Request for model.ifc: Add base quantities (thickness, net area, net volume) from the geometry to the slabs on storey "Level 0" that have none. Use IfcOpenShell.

First a look at what the model holds.

```python
import ifcopenshell
import ifcopenshell.util.element
import ifcopenshell.util.unit

model = ifcopenshell.open("model.ifc")
print(model.schema)
for unit_type in ("LENGTHUNIT", "AREAUNIT", "VOLUMEUNIT"):
    print(unit_type, ifcopenshell.util.unit.calculate_unit_scale(model, unit_type))
storey = next(s for s in model.by_type("IfcBuildingStorey") if s.Name == "Level 0")
slabs = [e for e in ifcopenshell.util.element.get_decomposition(storey) if e.is_a("IfcSlab")]
for e in sorted(slabs, key=lambda e: e.id()):
    print(e.id(), e.is_a(), e.Name, list(ifcopenshell.util.element.get_psets(e, qtos_only=True)), sep=" | ")
```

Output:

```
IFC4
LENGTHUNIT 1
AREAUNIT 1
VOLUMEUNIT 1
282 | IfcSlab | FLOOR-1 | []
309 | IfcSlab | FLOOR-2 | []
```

```python
import ifcopenshell
import ifcopenshell.api.pset
import ifcopenshell.geom
import ifcopenshell.util.element
import ifcopenshell.util.shape
import ifcopenshell.util.unit

model = ifcopenshell.open("model.ifc")
unit_scale = ifcopenshell.util.unit.calculate_unit_scale(model)
area_scale = ifcopenshell.util.unit.calculate_unit_scale(model, "AREAUNIT")
volume_scale = ifcopenshell.util.unit.calculate_unit_scale(model, "VOLUMEUNIT")
settings = ifcopenshell.geom.settings()

storey = next(s for s in model.by_type("IfcBuildingStorey") if s.Name == "Level 0")
slabs = [e for e in ifcopenshell.util.element.get_decomposition(storey) if e.is_a("IfcSlab")]

for e in sorted(slabs, key=lambda e: e.id()):
    if ifcopenshell.util.element.get_psets(e, qtos_only=True, should_inherit=False):
        continue
    # Geometry comes back in metres, in the element's own axes.
    shape = ifcopenshell.geom.create_shape(settings, e)
    values = {
        "Width": ifcopenshell.util.shape.get_z(shape.geometry) / unit_scale,
        "NetArea": ifcopenshell.util.shape.get_footprint_area(shape.geometry) / area_scale,
        "NetVolume": ifcopenshell.util.shape.get_volume(shape.geometry) / volume_scale,
    }
    qto = ifcopenshell.api.pset.add_qto(model, product=e, name="Qto_SlabBaseQuantities")
    ifcopenshell.api.pset.edit_qto(model, qto=qto, properties=values)
    print(e.id(), {k: round(v, 3) for k, v in values.items()})

model.write("model_rev.ifc")
```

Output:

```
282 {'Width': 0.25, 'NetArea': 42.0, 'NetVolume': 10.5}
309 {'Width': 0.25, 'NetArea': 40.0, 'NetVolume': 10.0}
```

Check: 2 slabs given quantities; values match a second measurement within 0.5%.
